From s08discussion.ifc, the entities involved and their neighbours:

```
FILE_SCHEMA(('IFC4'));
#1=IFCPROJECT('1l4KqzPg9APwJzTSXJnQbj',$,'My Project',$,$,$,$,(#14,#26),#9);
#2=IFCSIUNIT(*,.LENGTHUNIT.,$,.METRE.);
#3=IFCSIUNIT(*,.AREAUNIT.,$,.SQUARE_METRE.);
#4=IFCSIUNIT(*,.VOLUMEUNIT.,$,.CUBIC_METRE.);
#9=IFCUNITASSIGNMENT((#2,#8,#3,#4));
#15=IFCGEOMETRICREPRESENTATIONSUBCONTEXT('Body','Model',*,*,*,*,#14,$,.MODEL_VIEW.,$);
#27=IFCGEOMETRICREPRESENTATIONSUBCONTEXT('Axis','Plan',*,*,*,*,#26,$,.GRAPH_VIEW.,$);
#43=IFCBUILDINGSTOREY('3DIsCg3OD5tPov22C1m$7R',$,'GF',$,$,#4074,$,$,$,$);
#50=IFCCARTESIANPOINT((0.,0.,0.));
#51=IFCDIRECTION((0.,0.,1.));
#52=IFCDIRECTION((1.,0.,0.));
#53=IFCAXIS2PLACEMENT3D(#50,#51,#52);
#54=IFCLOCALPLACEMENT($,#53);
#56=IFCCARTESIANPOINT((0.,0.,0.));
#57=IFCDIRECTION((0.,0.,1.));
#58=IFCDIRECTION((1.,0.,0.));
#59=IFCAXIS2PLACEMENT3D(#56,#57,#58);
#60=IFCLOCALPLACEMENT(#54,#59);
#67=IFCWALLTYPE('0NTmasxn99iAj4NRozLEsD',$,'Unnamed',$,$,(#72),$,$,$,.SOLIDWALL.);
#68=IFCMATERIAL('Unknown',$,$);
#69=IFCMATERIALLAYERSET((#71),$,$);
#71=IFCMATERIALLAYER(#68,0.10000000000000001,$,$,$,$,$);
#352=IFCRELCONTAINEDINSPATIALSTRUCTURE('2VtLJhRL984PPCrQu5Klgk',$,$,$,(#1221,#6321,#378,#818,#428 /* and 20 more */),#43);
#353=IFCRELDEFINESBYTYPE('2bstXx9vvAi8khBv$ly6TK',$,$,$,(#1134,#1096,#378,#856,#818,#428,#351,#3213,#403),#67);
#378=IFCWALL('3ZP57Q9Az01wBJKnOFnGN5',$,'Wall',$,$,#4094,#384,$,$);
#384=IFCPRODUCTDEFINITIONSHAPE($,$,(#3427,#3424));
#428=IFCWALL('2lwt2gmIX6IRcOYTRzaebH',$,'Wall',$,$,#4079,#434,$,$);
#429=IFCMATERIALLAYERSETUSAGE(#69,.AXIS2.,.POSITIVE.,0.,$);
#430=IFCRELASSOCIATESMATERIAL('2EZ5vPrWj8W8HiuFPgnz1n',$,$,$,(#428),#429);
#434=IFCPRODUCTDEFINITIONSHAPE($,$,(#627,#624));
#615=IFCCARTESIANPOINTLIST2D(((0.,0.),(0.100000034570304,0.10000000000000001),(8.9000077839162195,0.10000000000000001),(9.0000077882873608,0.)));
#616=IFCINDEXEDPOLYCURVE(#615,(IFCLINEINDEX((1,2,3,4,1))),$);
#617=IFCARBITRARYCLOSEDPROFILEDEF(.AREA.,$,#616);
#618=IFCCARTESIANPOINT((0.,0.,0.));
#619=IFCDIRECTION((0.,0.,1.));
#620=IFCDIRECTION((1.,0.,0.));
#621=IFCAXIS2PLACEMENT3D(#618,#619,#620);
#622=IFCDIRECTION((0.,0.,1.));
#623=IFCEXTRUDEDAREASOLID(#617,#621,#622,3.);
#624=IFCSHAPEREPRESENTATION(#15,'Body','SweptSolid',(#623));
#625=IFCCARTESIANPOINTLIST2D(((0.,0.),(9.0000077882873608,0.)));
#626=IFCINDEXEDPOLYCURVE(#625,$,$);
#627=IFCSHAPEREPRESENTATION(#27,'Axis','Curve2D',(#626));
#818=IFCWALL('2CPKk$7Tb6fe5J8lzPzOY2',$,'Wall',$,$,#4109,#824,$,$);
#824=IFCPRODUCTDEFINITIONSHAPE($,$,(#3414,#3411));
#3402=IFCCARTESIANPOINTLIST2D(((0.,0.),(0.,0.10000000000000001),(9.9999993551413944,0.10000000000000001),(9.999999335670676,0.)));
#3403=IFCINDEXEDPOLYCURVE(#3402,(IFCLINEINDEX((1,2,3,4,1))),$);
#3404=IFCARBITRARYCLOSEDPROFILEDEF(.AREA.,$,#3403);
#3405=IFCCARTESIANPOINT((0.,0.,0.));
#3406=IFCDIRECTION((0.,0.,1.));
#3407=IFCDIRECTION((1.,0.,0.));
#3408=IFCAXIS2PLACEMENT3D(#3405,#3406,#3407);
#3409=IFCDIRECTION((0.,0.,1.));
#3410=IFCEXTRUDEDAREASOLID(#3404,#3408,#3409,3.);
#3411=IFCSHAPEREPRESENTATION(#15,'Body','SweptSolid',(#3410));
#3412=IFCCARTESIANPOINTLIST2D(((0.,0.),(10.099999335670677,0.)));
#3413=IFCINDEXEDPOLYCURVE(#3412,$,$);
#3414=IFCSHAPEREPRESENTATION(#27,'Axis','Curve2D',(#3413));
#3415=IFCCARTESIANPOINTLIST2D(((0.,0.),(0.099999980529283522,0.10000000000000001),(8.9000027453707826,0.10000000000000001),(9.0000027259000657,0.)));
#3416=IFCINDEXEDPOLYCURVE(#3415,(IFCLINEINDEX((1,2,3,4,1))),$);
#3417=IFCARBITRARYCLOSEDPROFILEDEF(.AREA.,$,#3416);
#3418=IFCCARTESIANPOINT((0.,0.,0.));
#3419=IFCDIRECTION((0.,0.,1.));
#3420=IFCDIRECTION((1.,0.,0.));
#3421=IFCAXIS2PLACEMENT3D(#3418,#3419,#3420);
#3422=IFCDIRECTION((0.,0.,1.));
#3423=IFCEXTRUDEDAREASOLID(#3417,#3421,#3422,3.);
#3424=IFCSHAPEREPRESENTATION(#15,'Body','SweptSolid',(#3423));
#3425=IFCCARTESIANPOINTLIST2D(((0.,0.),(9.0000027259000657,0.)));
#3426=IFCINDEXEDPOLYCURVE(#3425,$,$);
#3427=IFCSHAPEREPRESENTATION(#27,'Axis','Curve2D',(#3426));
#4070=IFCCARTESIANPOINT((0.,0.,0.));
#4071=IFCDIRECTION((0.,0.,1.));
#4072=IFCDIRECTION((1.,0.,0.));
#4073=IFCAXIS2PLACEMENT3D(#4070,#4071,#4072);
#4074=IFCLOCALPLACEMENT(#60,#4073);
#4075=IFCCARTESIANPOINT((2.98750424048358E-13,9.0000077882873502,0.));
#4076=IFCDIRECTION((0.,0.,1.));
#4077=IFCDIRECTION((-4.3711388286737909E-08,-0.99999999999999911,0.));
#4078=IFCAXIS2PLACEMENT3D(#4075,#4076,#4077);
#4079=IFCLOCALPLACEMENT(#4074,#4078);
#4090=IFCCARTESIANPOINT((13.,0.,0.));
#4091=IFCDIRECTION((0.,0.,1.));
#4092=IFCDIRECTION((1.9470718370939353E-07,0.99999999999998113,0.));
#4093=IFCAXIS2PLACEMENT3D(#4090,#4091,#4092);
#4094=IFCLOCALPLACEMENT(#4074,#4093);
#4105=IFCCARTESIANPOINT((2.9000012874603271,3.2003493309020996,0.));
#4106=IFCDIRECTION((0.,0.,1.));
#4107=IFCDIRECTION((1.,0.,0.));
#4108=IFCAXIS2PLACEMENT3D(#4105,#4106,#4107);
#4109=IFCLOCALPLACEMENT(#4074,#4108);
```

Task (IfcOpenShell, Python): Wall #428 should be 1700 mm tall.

```python
import ifcopenshell
import ifcopenshell.geom
import ifcopenshell.util.representation
import ifcopenshell.util.shape
import ifcopenshell.util.unit

model = ifcopenshell.open("s08discussion.ifc")
unit_scale = ifcopenshell.util.unit.calculate_unit_scale(model)
settings = ifcopenshell.geom.settings()


def volume(element):
    """Net volume in cubic metres, openings subtracted."""
    shape = ifcopenshell.geom.create_shape(settings, element)
    return ifcopenshell.util.shape.get_volume(shape.geometry)


wall = model.by_id(428)
before = volume(wall)

body = ifcopenshell.util.representation.get_representation(wall, "Model", "Body")
solid = body.Items[0]
old_height = solid.Depth
solid.Depth = 1.7 / unit_scale
after = volume(wall)

print(f"height {old_height:g} -> {solid.Depth:g}, volume {before:.3f} -> {after:.3f} m3")

model.write("s08discussion_rev.ifc")
```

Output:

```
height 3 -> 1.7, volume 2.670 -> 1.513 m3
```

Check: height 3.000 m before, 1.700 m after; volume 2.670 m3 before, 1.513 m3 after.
